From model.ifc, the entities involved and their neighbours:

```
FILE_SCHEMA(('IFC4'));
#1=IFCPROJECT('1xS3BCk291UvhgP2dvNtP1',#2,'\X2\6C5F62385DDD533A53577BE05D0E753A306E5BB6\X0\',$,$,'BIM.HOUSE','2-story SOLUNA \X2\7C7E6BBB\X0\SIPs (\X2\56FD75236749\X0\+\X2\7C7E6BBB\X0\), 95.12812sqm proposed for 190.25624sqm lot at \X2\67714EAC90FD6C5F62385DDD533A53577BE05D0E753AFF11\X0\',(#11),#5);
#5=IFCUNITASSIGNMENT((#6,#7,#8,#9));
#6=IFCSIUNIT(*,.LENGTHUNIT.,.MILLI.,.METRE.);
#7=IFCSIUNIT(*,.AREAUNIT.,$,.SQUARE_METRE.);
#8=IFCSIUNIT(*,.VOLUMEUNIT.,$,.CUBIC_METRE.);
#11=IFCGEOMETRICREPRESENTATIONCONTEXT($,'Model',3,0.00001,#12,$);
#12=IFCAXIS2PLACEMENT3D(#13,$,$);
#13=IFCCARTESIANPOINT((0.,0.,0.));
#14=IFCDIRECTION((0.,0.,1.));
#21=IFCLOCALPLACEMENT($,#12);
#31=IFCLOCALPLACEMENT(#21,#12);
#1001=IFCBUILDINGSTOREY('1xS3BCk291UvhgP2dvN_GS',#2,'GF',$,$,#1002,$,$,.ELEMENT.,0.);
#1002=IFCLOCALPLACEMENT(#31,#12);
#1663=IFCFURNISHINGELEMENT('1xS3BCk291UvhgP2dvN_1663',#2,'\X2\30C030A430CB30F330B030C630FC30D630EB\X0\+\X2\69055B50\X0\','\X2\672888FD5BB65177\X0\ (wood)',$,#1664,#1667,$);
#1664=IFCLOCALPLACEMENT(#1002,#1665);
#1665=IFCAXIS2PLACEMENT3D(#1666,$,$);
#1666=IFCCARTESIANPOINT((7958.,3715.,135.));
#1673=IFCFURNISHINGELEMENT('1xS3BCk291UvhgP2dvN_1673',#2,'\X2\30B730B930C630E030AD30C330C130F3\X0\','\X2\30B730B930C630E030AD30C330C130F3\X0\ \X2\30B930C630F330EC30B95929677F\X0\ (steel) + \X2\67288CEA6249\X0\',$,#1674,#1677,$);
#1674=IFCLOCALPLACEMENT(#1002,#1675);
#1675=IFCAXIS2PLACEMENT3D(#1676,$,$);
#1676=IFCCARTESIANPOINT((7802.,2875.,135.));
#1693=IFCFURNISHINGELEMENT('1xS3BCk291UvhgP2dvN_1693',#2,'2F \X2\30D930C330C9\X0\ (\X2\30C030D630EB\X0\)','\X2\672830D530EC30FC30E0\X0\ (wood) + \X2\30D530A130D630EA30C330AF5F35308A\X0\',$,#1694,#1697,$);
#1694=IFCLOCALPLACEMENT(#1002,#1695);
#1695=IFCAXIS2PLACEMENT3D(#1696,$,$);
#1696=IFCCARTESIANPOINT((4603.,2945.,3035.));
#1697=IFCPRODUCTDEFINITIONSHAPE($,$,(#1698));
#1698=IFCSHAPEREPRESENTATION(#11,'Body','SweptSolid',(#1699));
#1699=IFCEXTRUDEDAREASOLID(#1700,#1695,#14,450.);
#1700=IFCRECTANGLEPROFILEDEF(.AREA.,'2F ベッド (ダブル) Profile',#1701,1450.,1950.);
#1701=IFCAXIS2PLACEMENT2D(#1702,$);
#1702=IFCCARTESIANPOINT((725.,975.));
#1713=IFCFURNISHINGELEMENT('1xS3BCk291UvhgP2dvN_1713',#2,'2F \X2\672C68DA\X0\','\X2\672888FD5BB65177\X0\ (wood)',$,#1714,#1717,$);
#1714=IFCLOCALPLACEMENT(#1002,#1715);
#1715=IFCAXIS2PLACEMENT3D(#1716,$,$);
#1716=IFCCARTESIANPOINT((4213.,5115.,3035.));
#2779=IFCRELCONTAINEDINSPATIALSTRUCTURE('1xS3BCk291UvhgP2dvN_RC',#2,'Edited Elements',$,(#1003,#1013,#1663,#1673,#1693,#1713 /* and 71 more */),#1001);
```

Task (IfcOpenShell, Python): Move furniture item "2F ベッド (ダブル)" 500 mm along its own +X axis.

```python
import ifcopenshell
import ifcopenshell.api.geometry
import ifcopenshell.util.placement
import ifcopenshell.util.unit

model = ifcopenshell.open("model.ifc")
unit_scale = ifcopenshell.util.unit.calculate_unit_scale(model)

item = model.by_id(1693)
matrix = ifcopenshell.util.placement.get_local_placement(item.ObjectPlacement)
matrix[:3, 3] += matrix[:3, 0] * 0.5 / unit_scale
ifcopenshell.api.geometry.edit_object_placement(model, product=item, matrix=matrix, is_si=False)

print(ifcopenshell.util.placement.get_local_placement(item.ObjectPlacement).round(3) + 0.0)

model.write("model-out.ifc")
```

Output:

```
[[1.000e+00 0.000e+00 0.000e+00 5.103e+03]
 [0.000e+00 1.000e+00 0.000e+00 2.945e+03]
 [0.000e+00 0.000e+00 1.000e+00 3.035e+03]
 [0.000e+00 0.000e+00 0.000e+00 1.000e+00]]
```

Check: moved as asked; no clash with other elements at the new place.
